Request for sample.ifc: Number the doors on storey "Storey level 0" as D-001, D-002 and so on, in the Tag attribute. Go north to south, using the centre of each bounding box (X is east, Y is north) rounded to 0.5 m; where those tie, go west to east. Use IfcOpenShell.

First a look at what the model holds.

```python
import ifcopenshell
import ifcopenshell.util.element
import ifcopenshell.util.placement

model = ifcopenshell.open("sample.ifc")
print(model.schema)
storey = next(s for s in model.by_type("IfcBuildingStorey") if s.Name == "Storey level 0")
doors = [e for e in ifcopenshell.util.element.get_decomposition(storey) if e.is_a("IfcDoor")]
for e in sorted(doors, key=lambda e: e.id()):
    origin = ifcopenshell.util.placement.get_local_placement(e.ObjectPlacement)[:3, 3]
    print(e.id(), e.Tag, e.Name, origin.round(2) + 0.0, sep=" | ")
```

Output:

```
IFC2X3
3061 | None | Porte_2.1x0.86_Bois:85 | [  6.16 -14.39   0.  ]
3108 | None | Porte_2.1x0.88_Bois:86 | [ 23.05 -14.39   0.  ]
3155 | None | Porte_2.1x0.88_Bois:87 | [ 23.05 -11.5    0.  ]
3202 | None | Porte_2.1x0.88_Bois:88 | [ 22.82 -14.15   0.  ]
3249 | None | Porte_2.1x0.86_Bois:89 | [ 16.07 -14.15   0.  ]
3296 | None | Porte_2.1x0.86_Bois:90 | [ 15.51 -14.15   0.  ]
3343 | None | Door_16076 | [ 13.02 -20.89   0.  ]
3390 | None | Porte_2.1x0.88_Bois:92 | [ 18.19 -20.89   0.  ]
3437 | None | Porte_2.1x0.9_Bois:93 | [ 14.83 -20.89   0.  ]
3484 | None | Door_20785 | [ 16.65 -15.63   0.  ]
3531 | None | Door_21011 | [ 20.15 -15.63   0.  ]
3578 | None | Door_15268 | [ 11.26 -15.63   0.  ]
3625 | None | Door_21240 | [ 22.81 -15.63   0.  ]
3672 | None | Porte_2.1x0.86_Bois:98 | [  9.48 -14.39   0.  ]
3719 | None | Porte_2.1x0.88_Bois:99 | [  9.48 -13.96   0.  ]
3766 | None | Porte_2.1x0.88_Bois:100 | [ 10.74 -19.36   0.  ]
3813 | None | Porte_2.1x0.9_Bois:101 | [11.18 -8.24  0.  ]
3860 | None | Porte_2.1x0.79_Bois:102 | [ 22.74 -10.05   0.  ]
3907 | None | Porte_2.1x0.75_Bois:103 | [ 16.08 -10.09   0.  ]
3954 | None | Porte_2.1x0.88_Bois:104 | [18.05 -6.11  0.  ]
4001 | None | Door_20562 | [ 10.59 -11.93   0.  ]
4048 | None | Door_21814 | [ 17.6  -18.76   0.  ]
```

```python
import ifcopenshell
import ifcopenshell.geom
import ifcopenshell.util.element
import ifcopenshell.util.shape

model = ifcopenshell.open("sample.ifc")
settings = ifcopenshell.geom.settings()
settings.set("use-world-coords", True)


def centre(element):
    shape = ifcopenshell.geom.create_shape(settings, element)
    return ifcopenshell.util.shape.get_bbox_centroid(shape.geometry)


storey = next(s for s in model.by_type("IfcBuildingStorey") if s.Name == "Storey level 0")
doors = [e for e in ifcopenshell.util.element.get_decomposition(storey) if e.is_a("IfcDoor")]

# Insertion points can sit at a corner or the storey origin, so sort by the geometry (in metres).
centres = {e: centre(e) for e in doors}
doors.sort(key=lambda e: (-round(centres[e][1] / 0.5), centres[e][0]))

for i, e in enumerate(doors, start=1):
    number = f"D-0{i:02d}"
    e.Tag = number
    print(e.id(), number)

model.write("sample_updated.ifc")
```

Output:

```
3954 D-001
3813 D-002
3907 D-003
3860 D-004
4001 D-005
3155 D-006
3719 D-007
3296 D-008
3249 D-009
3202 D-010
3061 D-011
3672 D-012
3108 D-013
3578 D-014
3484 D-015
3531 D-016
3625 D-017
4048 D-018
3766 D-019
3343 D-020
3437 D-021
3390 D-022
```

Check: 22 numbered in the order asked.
